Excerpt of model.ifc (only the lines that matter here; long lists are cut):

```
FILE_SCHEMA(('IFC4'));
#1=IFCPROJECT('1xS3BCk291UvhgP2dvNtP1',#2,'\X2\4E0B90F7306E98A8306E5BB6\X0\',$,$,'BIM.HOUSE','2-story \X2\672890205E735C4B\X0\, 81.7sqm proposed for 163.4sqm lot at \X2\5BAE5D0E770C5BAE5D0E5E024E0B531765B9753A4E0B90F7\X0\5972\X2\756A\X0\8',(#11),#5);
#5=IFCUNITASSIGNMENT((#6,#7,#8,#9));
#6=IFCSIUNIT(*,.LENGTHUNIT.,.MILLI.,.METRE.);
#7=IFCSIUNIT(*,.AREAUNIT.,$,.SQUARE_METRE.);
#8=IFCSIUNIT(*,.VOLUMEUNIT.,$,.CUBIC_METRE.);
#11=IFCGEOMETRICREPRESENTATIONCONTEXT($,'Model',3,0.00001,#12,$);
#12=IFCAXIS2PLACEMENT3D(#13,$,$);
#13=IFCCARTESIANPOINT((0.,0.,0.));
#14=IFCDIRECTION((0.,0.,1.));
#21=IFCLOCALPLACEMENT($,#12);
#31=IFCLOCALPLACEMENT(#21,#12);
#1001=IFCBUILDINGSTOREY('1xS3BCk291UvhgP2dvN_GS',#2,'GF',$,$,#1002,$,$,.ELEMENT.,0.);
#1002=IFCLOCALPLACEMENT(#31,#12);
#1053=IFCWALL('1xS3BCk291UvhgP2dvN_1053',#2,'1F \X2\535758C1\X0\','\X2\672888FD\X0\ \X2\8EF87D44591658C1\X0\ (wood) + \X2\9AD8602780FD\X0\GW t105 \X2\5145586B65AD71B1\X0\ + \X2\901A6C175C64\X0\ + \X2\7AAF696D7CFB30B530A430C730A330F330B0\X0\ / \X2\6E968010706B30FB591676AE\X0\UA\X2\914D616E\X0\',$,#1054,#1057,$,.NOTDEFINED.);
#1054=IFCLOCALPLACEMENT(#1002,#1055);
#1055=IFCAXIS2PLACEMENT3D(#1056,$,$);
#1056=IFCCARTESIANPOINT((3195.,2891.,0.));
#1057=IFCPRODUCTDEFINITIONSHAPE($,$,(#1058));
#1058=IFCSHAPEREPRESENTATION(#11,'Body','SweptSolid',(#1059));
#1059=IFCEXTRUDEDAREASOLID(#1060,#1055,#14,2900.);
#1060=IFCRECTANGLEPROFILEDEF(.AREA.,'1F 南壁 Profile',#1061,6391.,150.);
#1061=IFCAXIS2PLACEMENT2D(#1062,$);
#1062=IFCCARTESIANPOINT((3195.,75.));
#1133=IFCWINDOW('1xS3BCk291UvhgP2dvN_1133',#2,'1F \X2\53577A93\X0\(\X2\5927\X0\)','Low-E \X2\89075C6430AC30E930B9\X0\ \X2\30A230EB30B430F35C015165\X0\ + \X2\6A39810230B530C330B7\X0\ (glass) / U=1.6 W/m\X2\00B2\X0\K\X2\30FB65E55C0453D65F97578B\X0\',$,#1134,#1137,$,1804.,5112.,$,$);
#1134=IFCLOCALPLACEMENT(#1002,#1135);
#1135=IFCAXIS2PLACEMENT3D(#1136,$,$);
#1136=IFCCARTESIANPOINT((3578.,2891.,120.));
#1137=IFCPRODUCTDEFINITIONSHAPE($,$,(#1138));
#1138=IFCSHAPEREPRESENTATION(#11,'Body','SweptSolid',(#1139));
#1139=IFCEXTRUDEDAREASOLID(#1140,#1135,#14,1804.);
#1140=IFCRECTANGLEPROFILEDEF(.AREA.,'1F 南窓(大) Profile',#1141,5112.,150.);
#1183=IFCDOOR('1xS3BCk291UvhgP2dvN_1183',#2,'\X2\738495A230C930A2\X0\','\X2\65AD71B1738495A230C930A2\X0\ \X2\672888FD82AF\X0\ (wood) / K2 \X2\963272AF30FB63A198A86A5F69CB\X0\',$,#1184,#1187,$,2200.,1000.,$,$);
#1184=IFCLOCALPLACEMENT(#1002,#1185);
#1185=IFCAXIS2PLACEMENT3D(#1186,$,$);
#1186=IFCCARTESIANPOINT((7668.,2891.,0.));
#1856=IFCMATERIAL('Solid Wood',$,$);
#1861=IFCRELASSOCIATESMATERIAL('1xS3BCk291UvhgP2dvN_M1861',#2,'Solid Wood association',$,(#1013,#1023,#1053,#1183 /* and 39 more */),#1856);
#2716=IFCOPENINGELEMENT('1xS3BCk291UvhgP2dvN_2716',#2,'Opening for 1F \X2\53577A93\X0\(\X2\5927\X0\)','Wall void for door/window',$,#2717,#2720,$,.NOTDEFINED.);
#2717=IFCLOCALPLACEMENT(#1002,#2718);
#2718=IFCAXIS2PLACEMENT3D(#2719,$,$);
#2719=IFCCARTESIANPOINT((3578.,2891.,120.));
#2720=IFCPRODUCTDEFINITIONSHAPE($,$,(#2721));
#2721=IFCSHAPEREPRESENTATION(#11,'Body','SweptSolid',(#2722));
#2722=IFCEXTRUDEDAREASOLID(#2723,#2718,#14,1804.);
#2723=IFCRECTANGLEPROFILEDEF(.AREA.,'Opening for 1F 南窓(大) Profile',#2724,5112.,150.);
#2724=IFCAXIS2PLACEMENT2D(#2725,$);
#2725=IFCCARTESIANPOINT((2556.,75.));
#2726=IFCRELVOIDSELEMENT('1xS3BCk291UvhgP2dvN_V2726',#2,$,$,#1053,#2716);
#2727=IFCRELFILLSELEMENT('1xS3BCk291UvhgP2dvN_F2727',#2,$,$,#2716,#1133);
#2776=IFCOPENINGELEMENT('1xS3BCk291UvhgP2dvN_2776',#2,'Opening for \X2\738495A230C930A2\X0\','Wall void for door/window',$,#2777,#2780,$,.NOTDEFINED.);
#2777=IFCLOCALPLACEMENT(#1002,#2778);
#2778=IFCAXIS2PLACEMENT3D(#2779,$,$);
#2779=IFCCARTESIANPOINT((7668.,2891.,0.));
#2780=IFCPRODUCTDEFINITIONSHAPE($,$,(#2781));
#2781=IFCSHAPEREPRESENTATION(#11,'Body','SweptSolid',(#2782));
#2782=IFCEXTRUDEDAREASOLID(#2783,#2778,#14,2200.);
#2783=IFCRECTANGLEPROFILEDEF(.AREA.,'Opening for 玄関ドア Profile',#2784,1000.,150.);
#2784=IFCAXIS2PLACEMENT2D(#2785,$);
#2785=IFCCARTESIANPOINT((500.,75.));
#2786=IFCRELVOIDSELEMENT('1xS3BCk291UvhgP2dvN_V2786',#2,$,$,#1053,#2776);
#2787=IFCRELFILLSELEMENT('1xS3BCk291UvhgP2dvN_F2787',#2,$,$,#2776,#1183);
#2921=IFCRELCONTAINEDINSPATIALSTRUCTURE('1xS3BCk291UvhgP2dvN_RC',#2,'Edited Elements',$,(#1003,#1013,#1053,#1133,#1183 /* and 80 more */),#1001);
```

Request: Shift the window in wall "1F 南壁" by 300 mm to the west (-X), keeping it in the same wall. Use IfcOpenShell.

```python
import ifcopenshell
import ifcopenshell.api.geometry
import ifcopenshell.util.placement
import ifcopenshell.util.unit

model = ifcopenshell.open("model.ifc")
unit_scale = ifcopenshell.util.unit.calculate_unit_scale(model)

window = model.by_id(1133)
opening = window.FillsVoids[0].RelatingOpeningElement
wall = opening.VoidsElements[0].RelatingBuildingElement

wall_matrix = ifcopenshell.util.placement.get_local_placement(wall.ObjectPlacement)
shift = wall_matrix[:3, 0] * -0.3 / unit_scale
before = ifcopenshell.util.placement.get_local_placement(window.ObjectPlacement)[:3, 3].copy()

# The window is not placed relative to its opening, so move both.
for product in (opening, window):
    matrix = ifcopenshell.util.placement.get_local_placement(product.ObjectPlacement)
    matrix[:3, 3] += shift
    ifcopenshell.api.geometry.edit_object_placement(model, product=product, matrix=matrix, is_si=False)

after = ifcopenshell.util.placement.get_local_placement(window.ObjectPlacement)[:3, 3]
print("window moved by", (after - before).round(3) + 0.0)

model.write("model_edited.ifc")
```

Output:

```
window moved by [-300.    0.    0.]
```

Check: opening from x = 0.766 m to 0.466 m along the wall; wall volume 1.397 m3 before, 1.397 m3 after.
